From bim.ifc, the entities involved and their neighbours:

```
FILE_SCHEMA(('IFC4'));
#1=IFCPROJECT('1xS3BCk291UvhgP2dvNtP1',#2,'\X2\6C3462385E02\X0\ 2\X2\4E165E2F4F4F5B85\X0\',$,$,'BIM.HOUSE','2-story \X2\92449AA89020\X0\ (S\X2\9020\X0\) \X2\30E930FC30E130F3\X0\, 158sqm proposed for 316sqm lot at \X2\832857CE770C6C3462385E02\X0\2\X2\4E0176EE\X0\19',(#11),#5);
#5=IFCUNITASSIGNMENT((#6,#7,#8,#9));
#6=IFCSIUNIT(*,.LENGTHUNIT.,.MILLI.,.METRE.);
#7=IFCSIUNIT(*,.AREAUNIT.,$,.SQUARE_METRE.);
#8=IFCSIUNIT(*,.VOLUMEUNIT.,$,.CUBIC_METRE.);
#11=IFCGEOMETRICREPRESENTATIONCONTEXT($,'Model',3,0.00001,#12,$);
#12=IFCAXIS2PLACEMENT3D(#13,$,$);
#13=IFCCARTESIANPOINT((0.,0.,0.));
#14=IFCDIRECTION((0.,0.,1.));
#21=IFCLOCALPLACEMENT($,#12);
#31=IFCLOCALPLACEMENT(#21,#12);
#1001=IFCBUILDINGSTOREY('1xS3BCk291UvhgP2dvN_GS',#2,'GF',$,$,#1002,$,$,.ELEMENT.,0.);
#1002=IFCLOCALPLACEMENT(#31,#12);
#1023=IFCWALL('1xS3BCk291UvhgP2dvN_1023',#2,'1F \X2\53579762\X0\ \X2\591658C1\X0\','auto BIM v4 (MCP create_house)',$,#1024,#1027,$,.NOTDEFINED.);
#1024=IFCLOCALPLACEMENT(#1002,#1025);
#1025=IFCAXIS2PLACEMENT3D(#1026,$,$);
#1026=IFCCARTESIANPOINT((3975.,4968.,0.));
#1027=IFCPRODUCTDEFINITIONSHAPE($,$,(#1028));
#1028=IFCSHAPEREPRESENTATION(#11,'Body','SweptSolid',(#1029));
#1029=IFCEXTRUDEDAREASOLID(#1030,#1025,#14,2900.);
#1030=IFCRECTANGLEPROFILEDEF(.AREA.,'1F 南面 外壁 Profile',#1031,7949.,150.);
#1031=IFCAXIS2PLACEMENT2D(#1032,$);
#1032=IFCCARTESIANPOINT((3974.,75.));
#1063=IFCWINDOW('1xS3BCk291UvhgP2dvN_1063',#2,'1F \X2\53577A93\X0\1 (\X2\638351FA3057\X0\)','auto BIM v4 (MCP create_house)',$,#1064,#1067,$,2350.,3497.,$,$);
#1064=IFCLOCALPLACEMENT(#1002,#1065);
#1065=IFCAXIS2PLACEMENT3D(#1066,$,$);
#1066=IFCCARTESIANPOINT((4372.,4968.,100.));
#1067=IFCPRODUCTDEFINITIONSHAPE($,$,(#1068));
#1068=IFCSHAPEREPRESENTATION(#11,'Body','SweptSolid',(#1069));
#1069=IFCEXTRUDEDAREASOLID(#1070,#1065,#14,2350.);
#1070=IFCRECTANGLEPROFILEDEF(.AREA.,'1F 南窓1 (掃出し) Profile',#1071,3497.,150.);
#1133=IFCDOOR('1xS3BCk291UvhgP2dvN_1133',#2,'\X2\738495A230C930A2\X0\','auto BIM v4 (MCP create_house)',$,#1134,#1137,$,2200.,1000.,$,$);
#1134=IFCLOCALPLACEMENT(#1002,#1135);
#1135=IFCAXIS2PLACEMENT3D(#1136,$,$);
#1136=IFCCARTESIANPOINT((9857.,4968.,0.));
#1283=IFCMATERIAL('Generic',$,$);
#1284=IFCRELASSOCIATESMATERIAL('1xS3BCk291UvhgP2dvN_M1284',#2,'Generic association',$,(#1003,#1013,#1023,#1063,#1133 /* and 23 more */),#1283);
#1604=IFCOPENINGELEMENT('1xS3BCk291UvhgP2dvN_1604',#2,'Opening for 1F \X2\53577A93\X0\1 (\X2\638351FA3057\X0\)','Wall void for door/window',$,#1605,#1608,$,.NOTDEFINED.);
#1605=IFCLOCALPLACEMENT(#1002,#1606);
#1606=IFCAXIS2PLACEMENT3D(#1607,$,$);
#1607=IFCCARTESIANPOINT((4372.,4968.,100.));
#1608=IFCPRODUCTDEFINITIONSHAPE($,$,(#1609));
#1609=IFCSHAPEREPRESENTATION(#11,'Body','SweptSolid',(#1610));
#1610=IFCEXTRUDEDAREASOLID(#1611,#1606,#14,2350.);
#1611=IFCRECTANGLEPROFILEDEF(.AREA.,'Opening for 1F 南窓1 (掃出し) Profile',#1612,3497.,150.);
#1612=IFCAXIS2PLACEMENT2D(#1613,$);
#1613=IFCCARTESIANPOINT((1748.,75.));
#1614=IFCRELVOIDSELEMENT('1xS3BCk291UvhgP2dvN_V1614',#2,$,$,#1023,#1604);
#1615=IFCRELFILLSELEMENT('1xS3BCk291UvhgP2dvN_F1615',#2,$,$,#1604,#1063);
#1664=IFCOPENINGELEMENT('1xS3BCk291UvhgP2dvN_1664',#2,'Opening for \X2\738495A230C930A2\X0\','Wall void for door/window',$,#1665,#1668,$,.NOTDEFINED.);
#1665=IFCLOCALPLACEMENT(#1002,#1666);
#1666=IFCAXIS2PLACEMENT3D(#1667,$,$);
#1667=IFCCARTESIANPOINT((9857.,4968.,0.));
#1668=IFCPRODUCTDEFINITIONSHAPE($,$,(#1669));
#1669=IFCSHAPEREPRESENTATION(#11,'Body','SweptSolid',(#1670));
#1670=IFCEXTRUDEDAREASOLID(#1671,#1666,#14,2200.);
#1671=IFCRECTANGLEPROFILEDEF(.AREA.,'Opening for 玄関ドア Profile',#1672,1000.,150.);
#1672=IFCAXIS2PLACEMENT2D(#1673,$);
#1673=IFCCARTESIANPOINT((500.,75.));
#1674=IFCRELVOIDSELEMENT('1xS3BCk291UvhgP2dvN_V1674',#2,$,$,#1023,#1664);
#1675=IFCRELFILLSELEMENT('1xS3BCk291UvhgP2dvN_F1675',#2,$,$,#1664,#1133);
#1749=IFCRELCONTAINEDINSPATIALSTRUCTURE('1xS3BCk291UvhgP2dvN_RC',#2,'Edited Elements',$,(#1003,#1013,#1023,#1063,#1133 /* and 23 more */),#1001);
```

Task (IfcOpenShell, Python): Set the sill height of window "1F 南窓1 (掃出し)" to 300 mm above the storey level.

```python
import numpy as np
import ifcopenshell
import ifcopenshell.api.geometry
import ifcopenshell.geom
import ifcopenshell.util.element
import ifcopenshell.util.placement
import ifcopenshell.util.shape
import ifcopenshell.util.unit

model = ifcopenshell.open("bim.ifc")
unit_scale = ifcopenshell.util.unit.calculate_unit_scale(model)

window = model.by_guid("1xS3BCk291UvhgP2dvN_1063")
opening = window.FillsVoids[0].RelatingOpeningElement
storey = ifcopenshell.util.element.get_container(window, ifc_class="IfcBuildingStorey")
level = ifcopenshell.util.placement.get_local_placement(storey.ObjectPlacement)[2, 3]

# The opening's origin need not be at the sill, so measure its lowest point.
shape = ifcopenshell.geom.create_shape(ifcopenshell.geom.settings(), opening)
bottom = ifcopenshell.util.shape.get_shape_bottom_elevation(shape, shape.geometry) / unit_scale
dz = level + 0.3 / unit_scale - bottom

shift = np.array([0.0, 0.0, dz])
# The window is not placed relative to its opening, so move both.
for product in (opening, window):
    matrix = ifcopenshell.util.placement.get_local_placement(product.ObjectPlacement)
    matrix[:3, 3] += shift
    ifcopenshell.api.geometry.edit_object_placement(model, product=product, matrix=matrix, is_si=False)

print(f"moved by {dz * unit_scale:+.3f} m")

model.write("bim_v2.ifc")
```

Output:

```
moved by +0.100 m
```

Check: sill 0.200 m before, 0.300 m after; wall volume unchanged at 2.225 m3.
